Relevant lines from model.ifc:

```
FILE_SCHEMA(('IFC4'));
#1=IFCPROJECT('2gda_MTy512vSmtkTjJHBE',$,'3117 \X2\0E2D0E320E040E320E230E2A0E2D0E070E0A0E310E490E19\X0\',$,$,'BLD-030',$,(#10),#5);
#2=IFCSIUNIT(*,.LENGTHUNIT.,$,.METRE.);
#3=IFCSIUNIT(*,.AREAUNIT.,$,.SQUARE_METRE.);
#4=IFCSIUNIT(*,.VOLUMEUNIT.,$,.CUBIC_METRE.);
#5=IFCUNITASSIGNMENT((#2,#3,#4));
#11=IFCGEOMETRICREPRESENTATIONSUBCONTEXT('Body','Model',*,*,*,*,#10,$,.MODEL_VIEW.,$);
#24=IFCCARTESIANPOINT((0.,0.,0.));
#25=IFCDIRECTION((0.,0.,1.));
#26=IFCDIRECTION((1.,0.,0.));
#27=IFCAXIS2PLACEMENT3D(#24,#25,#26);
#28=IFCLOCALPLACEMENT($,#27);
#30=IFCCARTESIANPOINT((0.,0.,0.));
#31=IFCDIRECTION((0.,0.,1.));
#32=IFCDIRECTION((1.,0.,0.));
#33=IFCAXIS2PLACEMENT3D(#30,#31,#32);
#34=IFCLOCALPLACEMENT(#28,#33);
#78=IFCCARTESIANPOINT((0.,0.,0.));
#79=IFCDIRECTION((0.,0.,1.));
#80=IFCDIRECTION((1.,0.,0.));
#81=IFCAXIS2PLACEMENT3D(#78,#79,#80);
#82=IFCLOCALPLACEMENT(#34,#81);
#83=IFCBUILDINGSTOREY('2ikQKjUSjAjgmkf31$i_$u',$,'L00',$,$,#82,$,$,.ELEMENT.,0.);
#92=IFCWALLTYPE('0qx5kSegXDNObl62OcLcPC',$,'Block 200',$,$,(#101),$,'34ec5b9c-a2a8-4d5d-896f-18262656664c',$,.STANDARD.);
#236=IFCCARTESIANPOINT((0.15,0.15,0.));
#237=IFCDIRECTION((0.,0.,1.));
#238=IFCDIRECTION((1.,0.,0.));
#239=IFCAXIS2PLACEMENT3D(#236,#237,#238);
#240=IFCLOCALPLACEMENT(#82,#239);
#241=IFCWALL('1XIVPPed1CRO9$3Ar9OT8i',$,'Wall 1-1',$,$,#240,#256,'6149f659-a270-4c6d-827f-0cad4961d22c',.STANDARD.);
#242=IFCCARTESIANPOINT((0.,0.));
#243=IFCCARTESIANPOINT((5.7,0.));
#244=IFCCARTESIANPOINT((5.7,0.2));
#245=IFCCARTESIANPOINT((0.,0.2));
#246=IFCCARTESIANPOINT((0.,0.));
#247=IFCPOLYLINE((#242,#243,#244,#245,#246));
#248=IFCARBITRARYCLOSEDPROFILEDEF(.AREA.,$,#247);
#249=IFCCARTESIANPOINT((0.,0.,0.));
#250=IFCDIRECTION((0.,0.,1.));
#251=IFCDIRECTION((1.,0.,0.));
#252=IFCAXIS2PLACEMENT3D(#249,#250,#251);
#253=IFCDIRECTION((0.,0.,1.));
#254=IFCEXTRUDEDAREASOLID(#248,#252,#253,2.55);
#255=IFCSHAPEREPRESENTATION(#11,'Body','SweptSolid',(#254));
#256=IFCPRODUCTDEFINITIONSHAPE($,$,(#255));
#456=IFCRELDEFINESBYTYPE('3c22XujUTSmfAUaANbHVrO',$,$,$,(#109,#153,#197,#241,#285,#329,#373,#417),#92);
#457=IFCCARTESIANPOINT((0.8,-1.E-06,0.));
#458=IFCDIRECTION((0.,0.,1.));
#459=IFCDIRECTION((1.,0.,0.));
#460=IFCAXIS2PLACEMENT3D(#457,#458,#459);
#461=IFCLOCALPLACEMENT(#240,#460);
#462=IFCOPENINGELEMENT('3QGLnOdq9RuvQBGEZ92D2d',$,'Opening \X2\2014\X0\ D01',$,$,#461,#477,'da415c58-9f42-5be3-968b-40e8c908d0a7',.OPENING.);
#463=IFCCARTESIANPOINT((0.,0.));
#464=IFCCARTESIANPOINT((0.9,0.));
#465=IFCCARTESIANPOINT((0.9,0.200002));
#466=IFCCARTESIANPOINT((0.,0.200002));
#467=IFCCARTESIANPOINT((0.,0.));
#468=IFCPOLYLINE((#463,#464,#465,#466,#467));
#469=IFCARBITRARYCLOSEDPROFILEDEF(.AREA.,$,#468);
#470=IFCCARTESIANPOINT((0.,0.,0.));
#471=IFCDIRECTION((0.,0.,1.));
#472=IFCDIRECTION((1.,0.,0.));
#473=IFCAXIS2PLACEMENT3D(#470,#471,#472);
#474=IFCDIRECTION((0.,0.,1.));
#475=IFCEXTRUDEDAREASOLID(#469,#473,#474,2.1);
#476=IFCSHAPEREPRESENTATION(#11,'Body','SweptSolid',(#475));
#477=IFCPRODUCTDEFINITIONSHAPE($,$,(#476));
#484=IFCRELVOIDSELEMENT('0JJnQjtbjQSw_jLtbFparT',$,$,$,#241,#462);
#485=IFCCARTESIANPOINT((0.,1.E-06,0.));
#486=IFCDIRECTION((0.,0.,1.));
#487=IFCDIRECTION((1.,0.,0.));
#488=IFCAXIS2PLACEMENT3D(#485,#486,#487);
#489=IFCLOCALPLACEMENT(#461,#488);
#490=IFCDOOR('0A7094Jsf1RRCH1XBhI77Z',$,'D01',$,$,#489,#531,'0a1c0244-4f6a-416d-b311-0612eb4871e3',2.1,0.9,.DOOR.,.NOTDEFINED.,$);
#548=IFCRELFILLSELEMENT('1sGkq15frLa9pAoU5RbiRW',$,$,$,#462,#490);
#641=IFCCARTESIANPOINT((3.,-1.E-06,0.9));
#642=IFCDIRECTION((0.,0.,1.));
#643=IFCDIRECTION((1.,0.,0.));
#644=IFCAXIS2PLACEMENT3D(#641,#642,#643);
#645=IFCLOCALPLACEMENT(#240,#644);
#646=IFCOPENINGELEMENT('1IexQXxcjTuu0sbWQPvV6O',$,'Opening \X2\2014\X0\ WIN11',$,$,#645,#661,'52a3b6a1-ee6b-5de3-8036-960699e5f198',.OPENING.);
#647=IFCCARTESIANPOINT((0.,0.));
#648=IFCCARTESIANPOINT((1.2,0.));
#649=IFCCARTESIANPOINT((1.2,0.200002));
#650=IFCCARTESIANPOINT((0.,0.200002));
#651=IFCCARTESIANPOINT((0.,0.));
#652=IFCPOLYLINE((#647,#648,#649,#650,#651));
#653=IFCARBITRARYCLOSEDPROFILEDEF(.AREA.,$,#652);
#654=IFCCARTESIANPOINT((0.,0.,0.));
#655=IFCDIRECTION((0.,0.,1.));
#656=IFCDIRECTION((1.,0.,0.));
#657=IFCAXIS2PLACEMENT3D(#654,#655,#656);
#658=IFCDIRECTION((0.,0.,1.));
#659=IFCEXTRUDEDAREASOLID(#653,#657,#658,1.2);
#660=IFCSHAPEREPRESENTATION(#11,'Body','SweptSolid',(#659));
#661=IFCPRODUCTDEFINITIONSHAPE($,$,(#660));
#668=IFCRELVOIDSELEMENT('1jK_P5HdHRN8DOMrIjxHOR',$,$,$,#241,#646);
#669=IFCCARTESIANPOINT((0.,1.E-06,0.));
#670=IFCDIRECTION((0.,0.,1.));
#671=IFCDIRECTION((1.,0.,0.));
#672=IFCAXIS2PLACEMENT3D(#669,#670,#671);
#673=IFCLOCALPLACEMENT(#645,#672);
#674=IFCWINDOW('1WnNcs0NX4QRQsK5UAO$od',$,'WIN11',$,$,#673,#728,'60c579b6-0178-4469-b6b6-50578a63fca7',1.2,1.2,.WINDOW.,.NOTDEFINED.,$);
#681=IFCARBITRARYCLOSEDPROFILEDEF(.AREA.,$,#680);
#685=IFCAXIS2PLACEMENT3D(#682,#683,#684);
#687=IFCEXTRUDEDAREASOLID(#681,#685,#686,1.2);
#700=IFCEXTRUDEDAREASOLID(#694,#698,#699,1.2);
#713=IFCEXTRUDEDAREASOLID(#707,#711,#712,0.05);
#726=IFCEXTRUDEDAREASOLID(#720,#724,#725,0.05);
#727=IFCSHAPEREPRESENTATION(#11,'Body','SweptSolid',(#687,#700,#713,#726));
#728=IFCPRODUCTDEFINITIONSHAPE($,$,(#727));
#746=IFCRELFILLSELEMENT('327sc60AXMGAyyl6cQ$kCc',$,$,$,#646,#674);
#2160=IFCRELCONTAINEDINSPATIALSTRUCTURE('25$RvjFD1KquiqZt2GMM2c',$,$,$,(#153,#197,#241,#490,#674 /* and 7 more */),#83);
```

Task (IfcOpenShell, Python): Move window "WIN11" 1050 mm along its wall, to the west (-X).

```python
import ifcopenshell
import ifcopenshell.api.geometry
import ifcopenshell.util.placement
import ifcopenshell.util.unit

model = ifcopenshell.open("model.ifc")
unit_scale = ifcopenshell.util.unit.calculate_unit_scale(model)

window = model.by_guid("1WnNcs0NX4QRQsK5UAO$od")
opening = window.FillsVoids[0].RelatingOpeningElement
wall = opening.VoidsElements[0].RelatingBuildingElement

wall_matrix = ifcopenshell.util.placement.get_local_placement(wall.ObjectPlacement)
shift = wall_matrix[:3, 0] * -1.05 / unit_scale
before = ifcopenshell.util.placement.get_local_placement(window.ObjectPlacement)[:3, 3].copy()

# The window is placed relative to its opening, so it follows when the opening moves.
matrix = ifcopenshell.util.placement.get_local_placement(opening.ObjectPlacement)
matrix[:3, 3] += shift
ifcopenshell.api.geometry.edit_object_placement(
    model, product=opening, matrix=matrix, is_si=False, should_transform_children=True
)

after = ifcopenshell.util.placement.get_local_placement(window.ObjectPlacement)[:3, 3]
print("window moved by", (after - before).round(3) + 0.0)

model.write("model_edited.ifc")
```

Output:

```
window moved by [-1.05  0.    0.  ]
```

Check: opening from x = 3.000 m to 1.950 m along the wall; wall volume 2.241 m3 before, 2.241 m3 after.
